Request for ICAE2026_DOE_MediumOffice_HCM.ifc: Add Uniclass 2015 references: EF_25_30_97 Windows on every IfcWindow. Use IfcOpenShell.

First a look at what the model holds.

```python
import ifcopenshell

model = ifcopenshell.open("ICAE2026_DOE_MediumOffice_HCM.ifc")
print(model.schema)
print("classifications:", [c.Name for c in model.by_type("IfcClassification")])
for ifc_class in ("IfcDoor", "IfcRoof", "IfcStair", "IfcWall", "IfcWindow"):
    print(ifc_class, len(model.by_type(ifc_class)))
```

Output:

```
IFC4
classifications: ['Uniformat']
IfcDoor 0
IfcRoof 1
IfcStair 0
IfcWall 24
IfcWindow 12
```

```python
import ifcopenshell
import ifcopenshell.api.classification

model = ifcopenshell.open("ICAE2026_DOE_MediumOffice_HCM.ifc")

system = ifcopenshell.api.classification.add_classification(model, classification="Uniclass 2015")

codes = {
    "IfcWindow": ("EF_25_30_97", "Windows"),
}
for ifc_class, (code, name) in codes.items():
    products = model.by_type(ifc_class)
    ifcopenshell.api.classification.add_reference(
        model, products=products, classification=system, identification=code, name=name
    )
    print(code, len(products))

model.write("ICAE2026_DOE_MediumOffice_HCM_edited.ifc")
```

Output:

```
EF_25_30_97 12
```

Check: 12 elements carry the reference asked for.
